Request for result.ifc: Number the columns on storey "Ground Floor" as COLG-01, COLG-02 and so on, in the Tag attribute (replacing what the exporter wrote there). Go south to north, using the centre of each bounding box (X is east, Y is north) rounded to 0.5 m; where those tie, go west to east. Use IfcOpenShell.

First a look at what the model holds.

```python
import ifcopenshell
import ifcopenshell.util.element
import ifcopenshell.util.placement

model = ifcopenshell.open("result.ifc")
print(model.schema)
storey = next(s for s in model.by_type("IfcBuildingStorey") if s.Name == "Ground Floor")
columns = [e for e in ifcopenshell.util.element.get_decomposition(storey) if e.is_a("IfcColumn")]
for e in sorted(columns, key=lambda e: e.id()):
    origin = ifcopenshell.util.placement.get_local_placement(e.ObjectPlacement)[:3, 3]
    print(e.id(), e.Tag, e.Name, origin.round(2) + 0.0, sep=" | ")
```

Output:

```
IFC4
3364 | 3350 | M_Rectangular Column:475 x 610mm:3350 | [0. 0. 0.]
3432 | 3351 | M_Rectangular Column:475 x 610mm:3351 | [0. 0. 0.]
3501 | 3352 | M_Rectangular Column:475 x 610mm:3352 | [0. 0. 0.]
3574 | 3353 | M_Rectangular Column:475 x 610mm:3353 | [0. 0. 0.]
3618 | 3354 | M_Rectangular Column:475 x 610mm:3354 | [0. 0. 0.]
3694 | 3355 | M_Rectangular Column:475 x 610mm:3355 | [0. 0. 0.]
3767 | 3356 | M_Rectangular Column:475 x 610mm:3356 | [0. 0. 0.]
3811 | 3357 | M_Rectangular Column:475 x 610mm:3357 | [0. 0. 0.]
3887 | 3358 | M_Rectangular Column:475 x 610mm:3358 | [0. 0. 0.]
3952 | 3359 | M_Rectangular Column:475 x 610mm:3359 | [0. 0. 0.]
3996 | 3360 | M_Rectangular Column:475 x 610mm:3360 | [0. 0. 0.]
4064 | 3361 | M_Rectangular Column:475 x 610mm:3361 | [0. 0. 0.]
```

```python
import ifcopenshell
import ifcopenshell.geom
import ifcopenshell.util.element
import ifcopenshell.util.shape

model = ifcopenshell.open("result.ifc")
settings = ifcopenshell.geom.settings()
settings.set("use-world-coords", True)


def centre(element):
    shape = ifcopenshell.geom.create_shape(settings, element)
    return ifcopenshell.util.shape.get_bbox_centroid(shape.geometry)


storey = next(s for s in model.by_type("IfcBuildingStorey") if s.Name == "Ground Floor")
columns = [e for e in ifcopenshell.util.element.get_decomposition(storey) if e.is_a("IfcColumn")]

# Insertion points can sit at a corner or the storey origin, so sort by the geometry (in metres).
centres = {e: centre(e) for e in columns}
columns.sort(key=lambda e: (round(centres[e][1] / 0.5), centres[e][0]))

for i, e in enumerate(columns, start=1):
    number = f"COLG-{i:02d}"
    e.Tag = number
    print(e.id(), number)

model.write("result_updated.ifc")
```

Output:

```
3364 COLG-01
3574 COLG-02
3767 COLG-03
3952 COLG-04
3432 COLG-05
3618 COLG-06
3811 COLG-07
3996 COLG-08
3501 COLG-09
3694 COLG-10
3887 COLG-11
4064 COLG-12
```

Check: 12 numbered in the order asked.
